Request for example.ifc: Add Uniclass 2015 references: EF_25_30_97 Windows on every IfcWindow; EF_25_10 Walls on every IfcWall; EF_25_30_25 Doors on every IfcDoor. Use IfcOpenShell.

First a look at what the model holds.

```python
import ifcopenshell

model = ifcopenshell.open("example.ifc")
print(model.schema)
print("classifications:", [c.Name for c in model.by_type("IfcClassification")])
for ifc_class in ("IfcDoor", "IfcRoof", "IfcStair", "IfcWall", "IfcWindow"):
    print(ifc_class, len(model.by_type(ifc_class)))
```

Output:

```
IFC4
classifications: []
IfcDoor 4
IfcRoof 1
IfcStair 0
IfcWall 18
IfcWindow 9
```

```python
import ifcopenshell
import ifcopenshell.api.classification

model = ifcopenshell.open("example.ifc")

system = ifcopenshell.api.classification.add_classification(model, classification="Uniclass 2015")

codes = {
    "IfcWindow": ("EF_25_30_97", "Windows"),
    "IfcWall": ("EF_25_10", "Walls"),
    "IfcDoor": ("EF_25_30_25", "Doors"),
}
for ifc_class, (code, name) in codes.items():
    products = model.by_type(ifc_class)
    ifcopenshell.api.classification.add_reference(
        model, products=products, classification=system, identification=code, name=name
    )
    print(code, len(products))

model.write("example_edited.ifc")
```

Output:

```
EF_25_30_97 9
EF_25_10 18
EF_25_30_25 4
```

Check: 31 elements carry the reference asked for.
